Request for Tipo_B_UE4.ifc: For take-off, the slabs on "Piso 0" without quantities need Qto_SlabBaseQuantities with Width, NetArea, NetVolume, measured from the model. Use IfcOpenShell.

First a look at what the model holds.

```python
import ifcopenshell
import ifcopenshell.util.element
import ifcopenshell.util.unit

model = ifcopenshell.open("Tipo_B_UE4.ifc")
print(model.schema)
for unit_type in ("LENGTHUNIT", "AREAUNIT", "VOLUMEUNIT"):
    print(unit_type, ifcopenshell.util.unit.calculate_unit_scale(model, unit_type))
storey = next(s for s in model.by_type("IfcBuildingStorey") if s.Name == "Piso 0")
slabs = [e for e in ifcopenshell.util.element.get_decomposition(storey) if e.is_a("IfcSlab")]
for e in sorted(slabs, key=lambda e: e.id()):
    print(e.id(), e.is_a(), e.Name, list(ifcopenshell.util.element.get_psets(e, qtos_only=True)), sep=" | ")
```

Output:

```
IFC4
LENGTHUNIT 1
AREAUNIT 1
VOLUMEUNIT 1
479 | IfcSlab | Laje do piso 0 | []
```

```python
import ifcopenshell
import ifcopenshell.api.pset
import ifcopenshell.geom
import ifcopenshell.util.element
import ifcopenshell.util.shape
import ifcopenshell.util.unit

model = ifcopenshell.open("Tipo_B_UE4.ifc")
unit_scale = ifcopenshell.util.unit.calculate_unit_scale(model)
area_scale = ifcopenshell.util.unit.calculate_unit_scale(model, "AREAUNIT")
volume_scale = ifcopenshell.util.unit.calculate_unit_scale(model, "VOLUMEUNIT")
settings = ifcopenshell.geom.settings()

storey = next(s for s in model.by_type("IfcBuildingStorey") if s.Name == "Piso 0")
slabs = [e for e in ifcopenshell.util.element.get_decomposition(storey) if e.is_a("IfcSlab")]

for e in sorted(slabs, key=lambda e: e.id()):
    if ifcopenshell.util.element.get_psets(e, qtos_only=True, should_inherit=False):
        continue
    # Geometry comes back in metres, in the element's own axes.
    shape = ifcopenshell.geom.create_shape(settings, e)
    values = {
        "Width": ifcopenshell.util.shape.get_z(shape.geometry) / unit_scale,
        "NetArea": ifcopenshell.util.shape.get_footprint_area(shape.geometry) / area_scale,
        "NetVolume": ifcopenshell.util.shape.get_volume(shape.geometry) / volume_scale,
    }
    qto = ifcopenshell.api.pset.add_qto(model, product=e, name="Qto_SlabBaseQuantities")
    ifcopenshell.api.pset.edit_qto(model, qto=qto, properties=values)
    print(e.id(), {k: round(v, 3) for k, v in values.items()})

model.write("Tipo_B_UE4-out.ifc")
```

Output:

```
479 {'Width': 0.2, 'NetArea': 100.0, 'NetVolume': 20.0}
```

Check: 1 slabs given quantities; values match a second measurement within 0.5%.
